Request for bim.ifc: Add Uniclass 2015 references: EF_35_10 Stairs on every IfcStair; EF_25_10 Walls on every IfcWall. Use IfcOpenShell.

First a look at what the model holds.

```python
import ifcopenshell

model = ifcopenshell.open("bim.ifc")
print(model.schema)
print("classifications:", [c.Name for c in model.by_type("IfcClassification")])
for ifc_class in ("IfcDoor", "IfcRoof", "IfcStair", "IfcWall", "IfcWindow"):
    print(ifc_class, len(model.by_type(ifc_class)))
```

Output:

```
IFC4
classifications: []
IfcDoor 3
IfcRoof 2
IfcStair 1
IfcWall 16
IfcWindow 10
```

```python
import ifcopenshell
import ifcopenshell.api.classification

model = ifcopenshell.open("bim.ifc")

system = ifcopenshell.api.classification.add_classification(model, classification="Uniclass 2015")

codes = {
    "IfcStair": ("EF_35_10", "Stairs"),
    "IfcWall": ("EF_25_10", "Walls"),
}
for ifc_class, (code, name) in codes.items():
    products = model.by_type(ifc_class)
    ifcopenshell.api.classification.add_reference(
        model, products=products, classification=system, identification=code, name=name
    )
    print(code, len(products))

model.write("bim_v2.ifc")
```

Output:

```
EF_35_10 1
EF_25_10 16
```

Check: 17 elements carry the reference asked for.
